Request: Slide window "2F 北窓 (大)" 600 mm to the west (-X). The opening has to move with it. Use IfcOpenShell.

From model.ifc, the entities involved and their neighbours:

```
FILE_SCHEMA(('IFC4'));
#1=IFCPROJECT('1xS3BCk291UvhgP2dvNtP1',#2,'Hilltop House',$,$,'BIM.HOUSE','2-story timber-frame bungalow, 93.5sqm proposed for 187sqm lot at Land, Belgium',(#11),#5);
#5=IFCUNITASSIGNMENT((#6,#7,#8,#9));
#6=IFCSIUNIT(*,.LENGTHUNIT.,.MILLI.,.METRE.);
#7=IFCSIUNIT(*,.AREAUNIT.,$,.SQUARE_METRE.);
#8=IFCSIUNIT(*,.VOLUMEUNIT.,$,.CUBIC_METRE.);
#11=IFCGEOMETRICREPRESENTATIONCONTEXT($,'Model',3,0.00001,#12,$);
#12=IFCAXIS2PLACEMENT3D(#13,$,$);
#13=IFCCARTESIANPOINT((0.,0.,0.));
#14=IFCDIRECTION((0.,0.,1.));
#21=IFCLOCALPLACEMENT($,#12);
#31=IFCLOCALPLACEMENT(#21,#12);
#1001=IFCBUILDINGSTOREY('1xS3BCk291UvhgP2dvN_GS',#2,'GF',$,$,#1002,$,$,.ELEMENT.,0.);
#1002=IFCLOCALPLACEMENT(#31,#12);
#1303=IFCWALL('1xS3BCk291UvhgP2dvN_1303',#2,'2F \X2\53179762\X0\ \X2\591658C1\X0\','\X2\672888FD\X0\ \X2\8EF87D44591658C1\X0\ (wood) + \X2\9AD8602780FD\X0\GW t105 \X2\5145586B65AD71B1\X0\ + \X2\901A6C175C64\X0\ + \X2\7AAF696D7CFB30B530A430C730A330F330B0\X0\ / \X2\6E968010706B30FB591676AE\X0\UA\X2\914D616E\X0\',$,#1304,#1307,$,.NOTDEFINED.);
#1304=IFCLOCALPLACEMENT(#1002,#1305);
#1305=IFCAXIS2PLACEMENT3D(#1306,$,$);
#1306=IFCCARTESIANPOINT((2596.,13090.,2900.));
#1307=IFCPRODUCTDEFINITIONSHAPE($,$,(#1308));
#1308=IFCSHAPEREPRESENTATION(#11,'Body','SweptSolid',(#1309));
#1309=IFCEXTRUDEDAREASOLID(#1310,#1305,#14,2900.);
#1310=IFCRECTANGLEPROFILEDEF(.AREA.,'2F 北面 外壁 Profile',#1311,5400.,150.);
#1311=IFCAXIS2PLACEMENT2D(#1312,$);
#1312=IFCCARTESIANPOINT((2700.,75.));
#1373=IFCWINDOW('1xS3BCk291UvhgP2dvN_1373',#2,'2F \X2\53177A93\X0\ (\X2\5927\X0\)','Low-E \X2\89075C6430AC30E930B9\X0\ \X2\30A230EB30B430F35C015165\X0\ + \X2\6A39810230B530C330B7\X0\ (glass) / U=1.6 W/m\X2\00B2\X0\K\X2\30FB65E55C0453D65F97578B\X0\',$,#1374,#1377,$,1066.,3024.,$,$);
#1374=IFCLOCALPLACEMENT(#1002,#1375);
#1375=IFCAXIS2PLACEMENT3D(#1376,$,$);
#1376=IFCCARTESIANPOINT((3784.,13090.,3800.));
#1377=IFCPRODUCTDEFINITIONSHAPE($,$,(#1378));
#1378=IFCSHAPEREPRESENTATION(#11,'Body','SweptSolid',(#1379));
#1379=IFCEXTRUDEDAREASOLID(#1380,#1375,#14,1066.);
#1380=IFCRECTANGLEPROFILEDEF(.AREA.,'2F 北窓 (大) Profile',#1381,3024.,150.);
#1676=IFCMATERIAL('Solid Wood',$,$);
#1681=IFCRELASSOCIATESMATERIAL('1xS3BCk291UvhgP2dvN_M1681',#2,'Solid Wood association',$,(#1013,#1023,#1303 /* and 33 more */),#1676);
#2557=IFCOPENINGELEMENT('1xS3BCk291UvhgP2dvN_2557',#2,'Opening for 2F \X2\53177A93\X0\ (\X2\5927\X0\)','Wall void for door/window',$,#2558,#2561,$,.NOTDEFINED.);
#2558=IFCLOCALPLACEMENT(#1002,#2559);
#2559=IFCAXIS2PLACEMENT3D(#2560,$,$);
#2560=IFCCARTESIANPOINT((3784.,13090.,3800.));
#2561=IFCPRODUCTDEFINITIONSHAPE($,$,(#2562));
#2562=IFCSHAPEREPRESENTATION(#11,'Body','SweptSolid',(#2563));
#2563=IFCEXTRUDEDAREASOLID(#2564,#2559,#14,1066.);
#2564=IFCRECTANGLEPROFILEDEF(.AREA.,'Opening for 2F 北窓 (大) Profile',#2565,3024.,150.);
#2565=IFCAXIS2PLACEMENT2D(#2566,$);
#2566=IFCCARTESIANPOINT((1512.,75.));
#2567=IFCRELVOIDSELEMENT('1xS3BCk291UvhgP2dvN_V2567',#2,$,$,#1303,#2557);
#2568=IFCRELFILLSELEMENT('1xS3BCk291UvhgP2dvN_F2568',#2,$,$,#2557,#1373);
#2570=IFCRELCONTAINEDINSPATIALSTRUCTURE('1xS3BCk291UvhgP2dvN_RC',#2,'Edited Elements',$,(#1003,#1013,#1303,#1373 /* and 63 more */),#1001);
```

```python
import ifcopenshell
import ifcopenshell.api.geometry
import ifcopenshell.util.placement
import ifcopenshell.util.unit

model = ifcopenshell.open("model.ifc")
unit_scale = ifcopenshell.util.unit.calculate_unit_scale(model)

window = model.by_guid("1xS3BCk291UvhgP2dvN_1373")
opening = window.FillsVoids[0].RelatingOpeningElement
wall = opening.VoidsElements[0].RelatingBuildingElement

wall_matrix = ifcopenshell.util.placement.get_local_placement(wall.ObjectPlacement)
shift = wall_matrix[:3, 0] * -0.6 / unit_scale
before = ifcopenshell.util.placement.get_local_placement(window.ObjectPlacement)[:3, 3].copy()

# The window is not placed relative to its opening, so move both.
for product in (opening, window):
    matrix = ifcopenshell.util.placement.get_local_placement(product.ObjectPlacement)
    matrix[:3, 3] += shift
    ifcopenshell.api.geometry.edit_object_placement(model, product=product, matrix=matrix, is_si=False)

after = ifcopenshell.util.placement.get_local_placement(window.ObjectPlacement)[:3, 3]
print("window moved by", (after - before).round(3) + 0.0)

model.write("model_updated.ifc")
```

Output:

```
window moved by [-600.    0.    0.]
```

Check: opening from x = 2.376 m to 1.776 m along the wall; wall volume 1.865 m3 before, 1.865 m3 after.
